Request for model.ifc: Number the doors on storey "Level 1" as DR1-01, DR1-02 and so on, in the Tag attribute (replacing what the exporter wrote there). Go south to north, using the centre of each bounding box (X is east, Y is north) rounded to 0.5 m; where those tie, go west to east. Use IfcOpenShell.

First a look at what the model holds.

```python
import ifcopenshell
import ifcopenshell.util.element
import ifcopenshell.util.placement

model = ifcopenshell.open("model.ifc")
print(model.schema)
storey = next(s for s in model.by_type("IfcBuildingStorey") if s.Name == "Level 1")
doors = [e for e in ifcopenshell.util.element.get_decomposition(storey) if e.is_a("IfcDoor")]
for e in sorted(doors, key=lambda e: e.id()):
    origin = ifcopenshell.util.placement.get_local_placement(e.ObjectPlacement)[:3, 3]
    print(e.id(), e.Tag, e.Name, origin.round(2) + 0.0, sep=" | ")
```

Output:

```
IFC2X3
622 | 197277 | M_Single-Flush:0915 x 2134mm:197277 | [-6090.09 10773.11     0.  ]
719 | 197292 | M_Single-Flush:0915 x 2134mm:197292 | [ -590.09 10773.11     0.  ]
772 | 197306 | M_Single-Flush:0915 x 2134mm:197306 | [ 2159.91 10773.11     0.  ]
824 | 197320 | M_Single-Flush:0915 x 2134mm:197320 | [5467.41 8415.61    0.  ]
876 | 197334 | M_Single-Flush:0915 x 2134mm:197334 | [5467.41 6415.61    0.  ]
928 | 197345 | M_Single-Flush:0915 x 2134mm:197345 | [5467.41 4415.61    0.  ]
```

```python
import ifcopenshell
import ifcopenshell.geom
import ifcopenshell.util.element
import ifcopenshell.util.shape

model = ifcopenshell.open("model.ifc")
settings = ifcopenshell.geom.settings()
settings.set("use-world-coords", True)


def centre(element):
    shape = ifcopenshell.geom.create_shape(settings, element)
    return ifcopenshell.util.shape.get_bbox_centroid(shape.geometry)


storey = next(s for s in model.by_type("IfcBuildingStorey") if s.Name == "Level 1")
doors = [e for e in ifcopenshell.util.element.get_decomposition(storey) if e.is_a("IfcDoor")]

# Insertion points can sit at a corner or the storey origin, so sort by the geometry (in metres).
centres = {e: centre(e) for e in doors}
doors.sort(key=lambda e: (round(centres[e][1] / 0.5), centres[e][0]))

for i, e in enumerate(doors, start=1):
    number = f"DR1-{i:02d}"
    e.Tag = number
    print(e.id(), number)

model.write("model_rev.ifc")
```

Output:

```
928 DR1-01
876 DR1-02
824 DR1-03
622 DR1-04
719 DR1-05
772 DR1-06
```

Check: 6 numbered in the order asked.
